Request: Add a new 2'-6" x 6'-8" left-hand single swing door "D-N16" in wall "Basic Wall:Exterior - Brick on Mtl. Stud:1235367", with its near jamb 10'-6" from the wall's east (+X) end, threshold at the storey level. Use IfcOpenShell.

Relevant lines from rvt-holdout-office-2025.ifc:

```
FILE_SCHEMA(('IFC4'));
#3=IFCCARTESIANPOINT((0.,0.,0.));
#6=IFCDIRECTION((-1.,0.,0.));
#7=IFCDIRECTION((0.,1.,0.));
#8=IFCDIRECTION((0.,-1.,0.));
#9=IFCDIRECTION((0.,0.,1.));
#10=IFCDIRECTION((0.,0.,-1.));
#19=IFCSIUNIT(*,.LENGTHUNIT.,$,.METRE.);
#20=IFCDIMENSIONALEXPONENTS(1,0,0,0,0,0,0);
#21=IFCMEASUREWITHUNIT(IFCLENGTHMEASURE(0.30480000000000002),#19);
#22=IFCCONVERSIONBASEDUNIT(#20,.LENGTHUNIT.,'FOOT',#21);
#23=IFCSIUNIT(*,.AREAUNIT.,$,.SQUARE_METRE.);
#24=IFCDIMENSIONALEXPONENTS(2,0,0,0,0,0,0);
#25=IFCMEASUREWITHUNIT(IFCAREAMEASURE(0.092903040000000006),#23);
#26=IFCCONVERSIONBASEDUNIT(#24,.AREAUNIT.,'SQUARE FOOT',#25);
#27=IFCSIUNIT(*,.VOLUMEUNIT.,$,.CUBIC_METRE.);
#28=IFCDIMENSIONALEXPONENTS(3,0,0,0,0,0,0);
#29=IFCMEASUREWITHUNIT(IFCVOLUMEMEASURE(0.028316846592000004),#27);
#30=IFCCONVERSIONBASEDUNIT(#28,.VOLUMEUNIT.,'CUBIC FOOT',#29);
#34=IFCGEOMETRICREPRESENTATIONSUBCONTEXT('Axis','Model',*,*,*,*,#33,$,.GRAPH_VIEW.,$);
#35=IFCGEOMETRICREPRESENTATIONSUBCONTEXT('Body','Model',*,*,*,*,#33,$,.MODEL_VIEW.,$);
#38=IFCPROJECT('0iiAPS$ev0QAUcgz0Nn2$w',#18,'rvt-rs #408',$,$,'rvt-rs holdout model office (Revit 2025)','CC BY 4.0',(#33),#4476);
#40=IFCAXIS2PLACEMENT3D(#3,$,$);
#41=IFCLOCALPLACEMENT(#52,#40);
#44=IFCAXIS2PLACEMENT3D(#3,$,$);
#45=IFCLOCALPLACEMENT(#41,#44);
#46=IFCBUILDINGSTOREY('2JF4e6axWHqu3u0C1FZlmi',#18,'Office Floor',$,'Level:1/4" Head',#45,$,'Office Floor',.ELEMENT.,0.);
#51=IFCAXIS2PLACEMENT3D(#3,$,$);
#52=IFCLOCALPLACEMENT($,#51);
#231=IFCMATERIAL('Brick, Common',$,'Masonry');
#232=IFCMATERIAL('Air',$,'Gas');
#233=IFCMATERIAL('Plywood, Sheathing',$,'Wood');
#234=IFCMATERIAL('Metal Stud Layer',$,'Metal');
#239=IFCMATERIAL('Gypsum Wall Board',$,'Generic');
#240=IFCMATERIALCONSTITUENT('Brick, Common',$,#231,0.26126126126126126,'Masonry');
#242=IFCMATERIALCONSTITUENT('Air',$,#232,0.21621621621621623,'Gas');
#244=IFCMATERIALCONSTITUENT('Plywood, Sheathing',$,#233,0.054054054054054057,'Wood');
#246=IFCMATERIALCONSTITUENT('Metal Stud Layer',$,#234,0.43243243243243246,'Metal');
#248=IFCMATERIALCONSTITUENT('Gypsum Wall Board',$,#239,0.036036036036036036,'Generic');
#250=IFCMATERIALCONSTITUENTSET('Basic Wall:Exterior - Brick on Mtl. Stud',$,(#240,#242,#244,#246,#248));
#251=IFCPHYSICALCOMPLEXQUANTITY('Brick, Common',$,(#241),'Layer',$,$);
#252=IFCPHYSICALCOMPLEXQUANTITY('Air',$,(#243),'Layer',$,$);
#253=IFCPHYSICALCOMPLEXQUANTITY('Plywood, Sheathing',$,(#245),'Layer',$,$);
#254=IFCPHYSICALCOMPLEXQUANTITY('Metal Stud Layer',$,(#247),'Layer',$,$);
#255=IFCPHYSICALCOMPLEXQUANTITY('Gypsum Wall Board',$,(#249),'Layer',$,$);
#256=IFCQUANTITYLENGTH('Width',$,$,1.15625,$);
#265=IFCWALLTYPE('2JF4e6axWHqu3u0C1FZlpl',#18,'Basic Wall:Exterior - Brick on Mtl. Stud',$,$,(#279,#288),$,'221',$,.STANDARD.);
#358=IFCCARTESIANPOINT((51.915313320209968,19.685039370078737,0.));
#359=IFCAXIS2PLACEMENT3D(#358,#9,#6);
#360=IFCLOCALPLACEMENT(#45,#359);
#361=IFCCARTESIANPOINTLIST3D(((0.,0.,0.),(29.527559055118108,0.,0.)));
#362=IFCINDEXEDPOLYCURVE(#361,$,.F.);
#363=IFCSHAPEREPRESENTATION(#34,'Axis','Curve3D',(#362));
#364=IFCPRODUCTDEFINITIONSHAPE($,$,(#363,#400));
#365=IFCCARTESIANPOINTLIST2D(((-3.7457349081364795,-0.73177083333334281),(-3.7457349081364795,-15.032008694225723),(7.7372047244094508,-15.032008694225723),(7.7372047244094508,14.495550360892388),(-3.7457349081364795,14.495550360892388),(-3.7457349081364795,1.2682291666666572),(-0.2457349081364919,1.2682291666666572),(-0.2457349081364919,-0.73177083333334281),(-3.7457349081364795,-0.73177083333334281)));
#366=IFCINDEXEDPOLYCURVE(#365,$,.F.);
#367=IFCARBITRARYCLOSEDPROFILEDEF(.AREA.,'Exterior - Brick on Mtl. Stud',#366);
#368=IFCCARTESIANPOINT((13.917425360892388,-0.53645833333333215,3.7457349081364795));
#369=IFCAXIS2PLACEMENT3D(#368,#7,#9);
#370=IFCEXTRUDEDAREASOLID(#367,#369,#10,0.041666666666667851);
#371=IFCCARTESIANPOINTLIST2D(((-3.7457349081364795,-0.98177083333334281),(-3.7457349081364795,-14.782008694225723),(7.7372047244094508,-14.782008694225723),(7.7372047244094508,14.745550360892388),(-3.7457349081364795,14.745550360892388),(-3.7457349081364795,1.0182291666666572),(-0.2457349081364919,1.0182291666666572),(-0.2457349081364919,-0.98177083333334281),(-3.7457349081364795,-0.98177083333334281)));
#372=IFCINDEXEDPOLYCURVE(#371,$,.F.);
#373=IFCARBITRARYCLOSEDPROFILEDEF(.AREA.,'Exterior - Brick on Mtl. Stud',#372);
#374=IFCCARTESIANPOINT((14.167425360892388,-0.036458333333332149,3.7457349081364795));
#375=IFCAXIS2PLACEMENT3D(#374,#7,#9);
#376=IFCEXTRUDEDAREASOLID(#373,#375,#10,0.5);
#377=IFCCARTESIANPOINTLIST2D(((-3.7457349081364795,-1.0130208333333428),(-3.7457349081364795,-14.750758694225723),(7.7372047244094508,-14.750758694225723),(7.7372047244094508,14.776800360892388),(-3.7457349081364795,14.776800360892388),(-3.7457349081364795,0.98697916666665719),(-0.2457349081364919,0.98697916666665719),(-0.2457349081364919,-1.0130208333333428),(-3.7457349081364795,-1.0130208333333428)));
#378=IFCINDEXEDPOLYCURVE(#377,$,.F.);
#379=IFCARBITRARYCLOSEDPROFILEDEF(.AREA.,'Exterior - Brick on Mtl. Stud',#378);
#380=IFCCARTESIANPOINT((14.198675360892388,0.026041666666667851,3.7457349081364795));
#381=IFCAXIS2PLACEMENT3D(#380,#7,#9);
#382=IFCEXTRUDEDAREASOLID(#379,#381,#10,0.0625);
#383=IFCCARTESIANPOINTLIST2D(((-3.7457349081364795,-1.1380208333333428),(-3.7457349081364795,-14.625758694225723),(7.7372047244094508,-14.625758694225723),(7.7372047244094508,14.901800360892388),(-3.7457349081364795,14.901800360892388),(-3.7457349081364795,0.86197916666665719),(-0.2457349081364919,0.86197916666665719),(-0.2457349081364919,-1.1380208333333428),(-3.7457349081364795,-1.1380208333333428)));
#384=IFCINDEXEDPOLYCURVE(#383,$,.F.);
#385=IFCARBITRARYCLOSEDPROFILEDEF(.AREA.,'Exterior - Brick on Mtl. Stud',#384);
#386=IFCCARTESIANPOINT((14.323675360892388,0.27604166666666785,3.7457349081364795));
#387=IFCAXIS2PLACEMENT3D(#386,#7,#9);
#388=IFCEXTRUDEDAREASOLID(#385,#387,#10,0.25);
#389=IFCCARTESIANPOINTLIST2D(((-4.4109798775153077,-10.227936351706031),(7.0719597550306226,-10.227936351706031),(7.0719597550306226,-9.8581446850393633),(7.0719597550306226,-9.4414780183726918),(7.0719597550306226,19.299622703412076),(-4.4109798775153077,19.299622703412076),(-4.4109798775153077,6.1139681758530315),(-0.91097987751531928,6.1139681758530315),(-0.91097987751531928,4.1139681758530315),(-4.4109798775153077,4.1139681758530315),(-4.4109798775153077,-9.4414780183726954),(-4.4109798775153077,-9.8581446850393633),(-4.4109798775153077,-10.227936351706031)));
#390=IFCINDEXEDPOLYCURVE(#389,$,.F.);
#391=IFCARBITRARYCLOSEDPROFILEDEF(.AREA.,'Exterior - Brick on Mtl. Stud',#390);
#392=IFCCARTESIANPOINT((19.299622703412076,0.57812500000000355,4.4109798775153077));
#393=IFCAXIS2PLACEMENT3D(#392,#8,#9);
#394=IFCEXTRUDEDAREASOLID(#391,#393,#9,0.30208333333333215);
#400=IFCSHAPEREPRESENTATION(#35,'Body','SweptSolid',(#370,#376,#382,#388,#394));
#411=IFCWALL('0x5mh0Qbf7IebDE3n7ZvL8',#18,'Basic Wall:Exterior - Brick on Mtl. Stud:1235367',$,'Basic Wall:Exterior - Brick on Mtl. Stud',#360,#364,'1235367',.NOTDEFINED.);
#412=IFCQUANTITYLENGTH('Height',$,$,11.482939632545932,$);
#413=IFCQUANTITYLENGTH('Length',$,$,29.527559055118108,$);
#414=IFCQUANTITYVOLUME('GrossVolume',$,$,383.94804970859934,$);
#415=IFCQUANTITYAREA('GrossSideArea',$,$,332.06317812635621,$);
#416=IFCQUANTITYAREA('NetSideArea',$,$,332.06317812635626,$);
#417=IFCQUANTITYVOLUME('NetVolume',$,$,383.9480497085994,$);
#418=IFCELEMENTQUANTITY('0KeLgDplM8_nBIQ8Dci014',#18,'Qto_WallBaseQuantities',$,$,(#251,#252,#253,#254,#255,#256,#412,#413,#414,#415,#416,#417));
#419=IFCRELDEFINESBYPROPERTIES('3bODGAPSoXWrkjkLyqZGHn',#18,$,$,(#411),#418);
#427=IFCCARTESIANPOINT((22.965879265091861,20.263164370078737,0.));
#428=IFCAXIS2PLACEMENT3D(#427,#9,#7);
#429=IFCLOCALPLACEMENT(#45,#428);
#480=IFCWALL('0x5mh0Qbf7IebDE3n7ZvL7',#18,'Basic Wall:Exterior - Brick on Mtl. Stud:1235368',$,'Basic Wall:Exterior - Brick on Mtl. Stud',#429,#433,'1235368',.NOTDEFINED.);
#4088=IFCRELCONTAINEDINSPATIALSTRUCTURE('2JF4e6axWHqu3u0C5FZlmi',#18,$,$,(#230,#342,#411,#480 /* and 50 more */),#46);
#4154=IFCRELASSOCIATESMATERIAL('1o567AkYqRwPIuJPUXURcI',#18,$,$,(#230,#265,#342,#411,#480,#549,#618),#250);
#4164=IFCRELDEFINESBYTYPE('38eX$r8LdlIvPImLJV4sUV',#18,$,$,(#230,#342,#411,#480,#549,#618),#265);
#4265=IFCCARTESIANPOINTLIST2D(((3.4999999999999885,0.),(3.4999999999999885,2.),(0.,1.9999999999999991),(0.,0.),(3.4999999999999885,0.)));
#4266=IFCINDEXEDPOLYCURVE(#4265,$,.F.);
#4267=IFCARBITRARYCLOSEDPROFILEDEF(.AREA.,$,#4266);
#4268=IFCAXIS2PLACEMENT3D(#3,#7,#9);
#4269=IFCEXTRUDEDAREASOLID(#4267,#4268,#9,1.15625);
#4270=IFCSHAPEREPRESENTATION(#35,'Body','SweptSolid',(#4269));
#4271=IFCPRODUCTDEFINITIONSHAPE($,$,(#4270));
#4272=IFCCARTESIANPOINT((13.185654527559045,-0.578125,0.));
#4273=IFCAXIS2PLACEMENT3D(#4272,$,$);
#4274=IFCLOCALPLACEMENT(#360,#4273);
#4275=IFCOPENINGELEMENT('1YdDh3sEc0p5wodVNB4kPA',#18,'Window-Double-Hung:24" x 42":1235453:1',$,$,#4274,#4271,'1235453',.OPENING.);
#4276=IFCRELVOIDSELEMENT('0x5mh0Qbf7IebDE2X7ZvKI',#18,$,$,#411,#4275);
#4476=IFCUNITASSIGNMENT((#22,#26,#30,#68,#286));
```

```python
import numpy as np
import ifcopenshell
import ifcopenshell.api.feature
import ifcopenshell.api.geometry
import ifcopenshell.api.pset
import ifcopenshell.api.root
import ifcopenshell.api.spatial
import ifcopenshell.geom
import ifcopenshell.util.element
import ifcopenshell.util.placement
import ifcopenshell.util.representation
import ifcopenshell.util.shape
import ifcopenshell.util.unit

model = ifcopenshell.open("rvt-holdout-office-2025.ifc")
unit_scale = ifcopenshell.util.unit.calculate_unit_scale(model)
area_scale = ifcopenshell.util.unit.calculate_unit_scale(model, "AREAUNIT")
volume_scale = ifcopenshell.util.unit.calculate_unit_scale(model, "VOLUMEUNIT")
settings = ifcopenshell.geom.settings()


def volume(element):
    """Net volume in cubic metres, openings subtracted."""
    shape = ifcopenshell.geom.create_shape(settings, element)
    return ifcopenshell.util.shape.get_volume(shape.geometry)


wall = model.by_id(411)
storey = ifcopenshell.util.element.get_container(wall, ifc_class="IfcBuildingStorey")
context = ifcopenshell.util.representation.get_context(model, "Model", "Body", "MODEL_VIEW")
before = volume(wall)

width, height, from_end, sill = 0.762, 2.032, 3.2004, 0.0  # metres

# The wall runs along its own X axis, and the end named is its -X end.
wall_shape = ifcopenshell.geom.create_shape(settings, wall)
x, y, z = ifcopenshell.util.shape.get_vertices(wall_shape.geometry).T
start = x.min() + from_end
face, thickness = float(y.min()), float(y.max() - y.min())
wall_matrix = ifcopenshell.util.placement.get_local_placement(wall.ObjectPlacement)
level = ifcopenshell.util.placement.get_local_placement(storey.ObjectPlacement)[2, 3]


def in_wall(x, y):
    """Placement at x, y metres in the wall's axes, at sill height."""
    matrix = wall_matrix.copy()
    matrix[:, 3] = wall_matrix @ np.array([x / unit_scale, y / unit_scale, 0.0, 1.0])
    matrix[2, 3] = level + sill / unit_scale
    return matrix


# Opening: a box that overshoots both wall faces by 50 mm.
opening = ifcopenshell.api.root.create_entity(model, ifc_class="IfcOpeningElement", predefined_type="OPENING")
box = ifcopenshell.api.geometry.add_wall_representation(
    model, context=context, length=width, height=height, thickness=thickness + 0.1
)
ifcopenshell.api.geometry.assign_representation(model, product=opening, representation=box)
ifcopenshell.api.geometry.edit_object_placement(model, product=opening, matrix=in_wall(start, face - 0.05), is_si=False)
ifcopenshell.api.feature.add_feature(model, feature=opening, element=wall)

door = ifcopenshell.api.root.create_entity(model, ifc_class="IfcDoor", name="D-N16", predefined_type="DOOR")
door.OverallWidth, door.OverallHeight = width / unit_scale, height / unit_scale
door.OperationType = "SINGLE_SWING_LEFT"
body = ifcopenshell.api.geometry.add_door_representation(
    model,
    context=context,
    overall_width=door.OverallWidth,
    overall_height=door.OverallHeight,
    operation_type="SINGLE_SWING_LEFT",
    lining_properties={"LiningDepth": thickness / unit_scale, "ThresholdDepth": thickness / unit_scale},
)
ifcopenshell.api.geometry.assign_representation(model, product=door, representation=body)
ifcopenshell.api.spatial.assign_container(model, products=[door], relating_structure=storey)
ifcopenshell.api.feature.add_filling(model, opening=opening, element=door)

# The lining spans the wall, so the door starts at the wall face.
ifcopenshell.api.geometry.edit_object_placement(model, product=door, matrix=in_wall(start, face), is_si=False)

after = volume(wall)

# Update the wall's stored quantities.
qto = model.by_id(ifcopenshell.util.element.get_pset(wall, "Qto_WallBaseQuantities", should_inherit=False)["id"])
ifcopenshell.api.pset.edit_qto(model, qto=qto, properties={
    "NetSideArea": after / thickness / area_scale,
    "NetVolume": after / volume_scale,
})

print(f"wall volume {before:.3f} -> {after:.3f} m3")

model.write("rvt-holdout-office-2025_updated.ifc")
```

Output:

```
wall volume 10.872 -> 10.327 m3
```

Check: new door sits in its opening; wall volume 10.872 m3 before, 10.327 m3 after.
